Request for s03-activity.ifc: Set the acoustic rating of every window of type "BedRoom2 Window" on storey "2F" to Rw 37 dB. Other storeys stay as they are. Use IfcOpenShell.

First a look at what the model holds.

```python
import ifcopenshell
import ifcopenshell.util.element

model = ifcopenshell.open("s03-activity.ifc")
print(model.schema)
storey = next(s for s in model.by_type("IfcBuildingStorey") if s.Name == "2F")
windows = [e for e in ifcopenshell.util.element.get_decomposition(storey) if e.is_a("IfcWindow")]
seen = {}
for e in windows:
    element_type = ifcopenshell.util.element.get_type(e)
    key = (element_type.Name if element_type != e and element_type else None, ifcopenshell.util.element.get_pset(e, "Pset_WindowCommon", "AcousticRating"))
    seen[key] = seen.get(key, 0) + 1
for (name, value), count in sorted(seen.items(), key=str):
    print(count, "x", name, "|", value)
```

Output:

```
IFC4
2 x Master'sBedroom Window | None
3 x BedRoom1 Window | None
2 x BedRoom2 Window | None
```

```python
import ifcopenshell
import ifcopenshell.api.pset
import ifcopenshell.util.element

model = ifcopenshell.open("s03-activity.ifc")

storey = next(s for s in model.by_type("IfcBuildingStorey") if s.Name == "2F")
windows = [e for e in ifcopenshell.util.element.get_decomposition(storey) if e.is_a("IfcWindow")]

count = 0
for e in windows:
    element_type = ifcopenshell.util.element.get_type(e)
    if element_type in (None, e) or element_type.Name != "BedRoom2 Window":
        continue
    # add_pset returns the element's existing set when there is one.
    pset = ifcopenshell.api.pset.add_pset(model, product=e, name="Pset_WindowCommon")
    ifcopenshell.api.pset.edit_pset(model, pset=pset, properties={"AcousticRating": "Rw 37 dB"})
    count += 1

print(count, "windows updated")

model.write("s03-activity-out.ifc")
```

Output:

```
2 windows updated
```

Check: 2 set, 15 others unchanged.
